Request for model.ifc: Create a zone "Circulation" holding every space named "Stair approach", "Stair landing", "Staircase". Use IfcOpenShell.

First a look at what the model holds.

```python
import ifcopenshell

model = ifcopenshell.open("model.ifc")
print(model.schema)
seen = {}
for space in model.by_type("IfcSpace"):
    seen[space.Name] = seen.get(space.Name, 0) + 1
for name, count in sorted(seen.items(), key=str):
    print(count, "x", name)
print("zones:", [z.Name for z in model.by_type("IfcZone")][:20])
```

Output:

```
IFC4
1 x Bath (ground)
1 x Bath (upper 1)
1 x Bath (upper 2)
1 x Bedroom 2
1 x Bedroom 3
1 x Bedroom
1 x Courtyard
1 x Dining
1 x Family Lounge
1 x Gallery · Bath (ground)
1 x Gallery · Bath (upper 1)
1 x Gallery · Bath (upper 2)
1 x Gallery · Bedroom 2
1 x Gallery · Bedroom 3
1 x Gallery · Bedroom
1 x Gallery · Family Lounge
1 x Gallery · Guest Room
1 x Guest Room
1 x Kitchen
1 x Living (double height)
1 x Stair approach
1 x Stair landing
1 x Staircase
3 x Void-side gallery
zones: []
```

```python
import ifcopenshell
import ifcopenshell.api.group
import ifcopenshell.api.root

model = ifcopenshell.open("model.ifc")

names = {"Stair approach", "Stair landing", "Staircase"}
spaces = [s for s in model.by_type("IfcSpace") if s.Name in names]

zone = ifcopenshell.api.root.create_entity(model, ifc_class="IfcZone", name="Circulation")
ifcopenshell.api.group.assign_group(model, products=spaces, group=zone)
print(len(spaces), "spaces in", zone.Name)

model.write("model_v2.ifc")
```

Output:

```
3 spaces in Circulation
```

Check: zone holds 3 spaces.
